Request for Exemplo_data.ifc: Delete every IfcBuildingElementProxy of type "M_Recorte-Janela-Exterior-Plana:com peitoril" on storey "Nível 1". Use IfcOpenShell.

First a look at what the model holds.

```python
import ifcopenshell
import ifcopenshell.util.element

model = ifcopenshell.open("Exemplo_data.ifc")
print(model.schema)
storey = next(s for s in model.by_type("IfcBuildingStorey") if s.Name == "Nível 1")
proxies = [e for e in ifcopenshell.util.element.get_decomposition(storey) if e.is_a("IfcBuildingElementProxy")]
seen = {}
for e in proxies:
    element_type = ifcopenshell.util.element.get_type(e)
    name = element_type.Name if element_type not in (None, e) else None
    seen[name] = seen.get(name, 0) + 1
for name, count in sorted(seen.items(), key=str):
    print(count, "x", name)
```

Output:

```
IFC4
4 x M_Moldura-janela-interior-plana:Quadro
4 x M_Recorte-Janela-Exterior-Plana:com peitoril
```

```python
import ifcopenshell
import ifcopenshell.api.root
import ifcopenshell.util.element

model = ifcopenshell.open("Exemplo_data.ifc")

storey = next(s for s in model.by_type("IfcBuildingStorey") if s.Name == "Nível 1")
proxies = [e for e in ifcopenshell.util.element.get_decomposition(storey) if e.is_a("IfcBuildingElementProxy")]
targets = [e for e in proxies if (t := ifcopenshell.util.element.get_type(e)) not in (None, e) and t.Name == "M_Recorte-Janela-Exterior-Plana:com peitoril"]

for e in targets:
    ifcopenshell.api.root.remove_product(model, product=e)
print(len(targets), "removed")

model.write("Exemplo_data_v2.ifc")
```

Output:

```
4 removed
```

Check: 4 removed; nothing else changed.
